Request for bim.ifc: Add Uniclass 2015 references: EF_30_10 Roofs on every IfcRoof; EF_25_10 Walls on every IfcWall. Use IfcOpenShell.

First a look at what the model holds.

```python
import ifcopenshell

model = ifcopenshell.open("bim.ifc")
print(model.schema)
print("classifications:", [c.Name for c in model.by_type("IfcClassification")])
for ifc_class in ("IfcDoor", "IfcRoof", "IfcStair", "IfcWall", "IfcWindow"):
    print(ifc_class, len(model.by_type(ifc_class)))
```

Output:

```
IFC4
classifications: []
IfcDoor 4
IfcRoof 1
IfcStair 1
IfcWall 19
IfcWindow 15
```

```python
import ifcopenshell
import ifcopenshell.api.classification

model = ifcopenshell.open("bim.ifc")

system = ifcopenshell.api.classification.add_classification(model, classification="Uniclass 2015")

codes = {
    "IfcRoof": ("EF_30_10", "Roofs"),
    "IfcWall": ("EF_25_10", "Walls"),
}
for ifc_class, (code, name) in codes.items():
    products = model.by_type(ifc_class)
    ifcopenshell.api.classification.add_reference(
        model, products=products, classification=system, identification=code, name=name
    )
    print(code, len(products))

model.write("bim-out.ifc")
```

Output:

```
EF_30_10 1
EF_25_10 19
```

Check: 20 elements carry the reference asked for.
